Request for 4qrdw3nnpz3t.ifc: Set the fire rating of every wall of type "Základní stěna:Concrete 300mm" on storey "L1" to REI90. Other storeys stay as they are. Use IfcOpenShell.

First a look at what the model holds.

```python
import ifcopenshell
import ifcopenshell.util.element

model = ifcopenshell.open("4qrdw3nnpz3t.ifc")
print(model.schema)
storey = next(s for s in model.by_type("IfcBuildingStorey") if s.Name == "L1")
walls = [e for e in ifcopenshell.util.element.get_decomposition(storey) if e.is_a("IfcWall")]
seen = {}
for e in walls:
    element_type = ifcopenshell.util.element.get_type(e)
    key = (element_type.Name if element_type != e and element_type else None, ifcopenshell.util.element.get_pset(e, "Pset_WallCommon", "FireRating"))
    seen[key] = seen.get(key, 0) + 1
for (name, value), count in sorted(seen.items(), key=str):
    print(count, "x", name, "|", value)
```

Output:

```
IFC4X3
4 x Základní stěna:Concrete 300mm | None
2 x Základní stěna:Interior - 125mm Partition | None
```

```python
import ifcopenshell
import ifcopenshell.api.pset
import ifcopenshell.util.element

model = ifcopenshell.open("4qrdw3nnpz3t.ifc")

storey = next(s for s in model.by_type("IfcBuildingStorey") if s.Name == "L1")
walls = [e for e in ifcopenshell.util.element.get_decomposition(storey) if e.is_a("IfcWall")]

count = 0
for e in walls:
    element_type = ifcopenshell.util.element.get_type(e)
    if element_type in (None, e) or element_type.Name != "Základní stěna:Concrete 300mm":
        continue
    # add_pset returns the element's existing set when there is one.
    pset = ifcopenshell.api.pset.add_pset(model, product=e, name="Pset_WallCommon")
    ifcopenshell.api.pset.edit_pset(model, pset=pset, properties={"FireRating": "REI90"})
    count += 1

print(count, "walls updated")

model.write("4qrdw3nnpz3t_v2.ifc")
```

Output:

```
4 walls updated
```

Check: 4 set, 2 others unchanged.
